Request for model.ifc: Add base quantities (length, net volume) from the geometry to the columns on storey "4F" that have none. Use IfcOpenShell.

First a look at what the model holds.

```python
import ifcopenshell
import ifcopenshell.util.element
import ifcopenshell.util.unit

model = ifcopenshell.open("model.ifc")
print(model.schema)
for unit_type in ("LENGTHUNIT", "AREAUNIT", "VOLUMEUNIT"):
    print(unit_type, ifcopenshell.util.unit.calculate_unit_scale(model, unit_type))
storey = next(s for s in model.by_type("IfcBuildingStorey") if s.Name == "4F")
columns = [e for e in ifcopenshell.util.element.get_decomposition(storey) if e.is_a("IfcColumn")]
for e in sorted(columns, key=lambda e: e.id()):
    print(e.id(), e.is_a(), e.Name, list(ifcopenshell.util.element.get_psets(e, qtos_only=True)), sep=" | ")
```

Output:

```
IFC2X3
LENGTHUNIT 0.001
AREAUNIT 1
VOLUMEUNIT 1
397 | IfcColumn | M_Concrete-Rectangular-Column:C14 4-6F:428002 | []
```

```python
import ifcopenshell
import ifcopenshell.api.pset
import ifcopenshell.geom
import ifcopenshell.util.element
import ifcopenshell.util.shape
import ifcopenshell.util.unit

model = ifcopenshell.open("model.ifc")
unit_scale = ifcopenshell.util.unit.calculate_unit_scale(model)
volume_scale = ifcopenshell.util.unit.calculate_unit_scale(model, "VOLUMEUNIT")
settings = ifcopenshell.geom.settings()

storey = next(s for s in model.by_type("IfcBuildingStorey") if s.Name == "4F")
columns = [e for e in ifcopenshell.util.element.get_decomposition(storey) if e.is_a("IfcColumn")]

for e in sorted(columns, key=lambda e: e.id()):
    if ifcopenshell.util.element.get_psets(e, qtos_only=True, should_inherit=False):
        continue
    # Geometry comes back in metres, in the element's own axes.
    shape = ifcopenshell.geom.create_shape(settings, e)
    values = {
        "Length": ifcopenshell.util.shape.get_z(shape.geometry) / unit_scale,
        "NetVolume": ifcopenshell.util.shape.get_volume(shape.geometry) / volume_scale,
    }
    qto = ifcopenshell.api.pset.add_qto(model, product=e, name="BaseQuantities")
    ifcopenshell.api.pset.edit_qto(model, qto=qto, properties=values)
    print(e.id(), {k: round(v, 3) for k, v in values.items()})

model.write("model_edited.ifc")
```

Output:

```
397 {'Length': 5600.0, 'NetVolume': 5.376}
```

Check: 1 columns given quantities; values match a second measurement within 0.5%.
